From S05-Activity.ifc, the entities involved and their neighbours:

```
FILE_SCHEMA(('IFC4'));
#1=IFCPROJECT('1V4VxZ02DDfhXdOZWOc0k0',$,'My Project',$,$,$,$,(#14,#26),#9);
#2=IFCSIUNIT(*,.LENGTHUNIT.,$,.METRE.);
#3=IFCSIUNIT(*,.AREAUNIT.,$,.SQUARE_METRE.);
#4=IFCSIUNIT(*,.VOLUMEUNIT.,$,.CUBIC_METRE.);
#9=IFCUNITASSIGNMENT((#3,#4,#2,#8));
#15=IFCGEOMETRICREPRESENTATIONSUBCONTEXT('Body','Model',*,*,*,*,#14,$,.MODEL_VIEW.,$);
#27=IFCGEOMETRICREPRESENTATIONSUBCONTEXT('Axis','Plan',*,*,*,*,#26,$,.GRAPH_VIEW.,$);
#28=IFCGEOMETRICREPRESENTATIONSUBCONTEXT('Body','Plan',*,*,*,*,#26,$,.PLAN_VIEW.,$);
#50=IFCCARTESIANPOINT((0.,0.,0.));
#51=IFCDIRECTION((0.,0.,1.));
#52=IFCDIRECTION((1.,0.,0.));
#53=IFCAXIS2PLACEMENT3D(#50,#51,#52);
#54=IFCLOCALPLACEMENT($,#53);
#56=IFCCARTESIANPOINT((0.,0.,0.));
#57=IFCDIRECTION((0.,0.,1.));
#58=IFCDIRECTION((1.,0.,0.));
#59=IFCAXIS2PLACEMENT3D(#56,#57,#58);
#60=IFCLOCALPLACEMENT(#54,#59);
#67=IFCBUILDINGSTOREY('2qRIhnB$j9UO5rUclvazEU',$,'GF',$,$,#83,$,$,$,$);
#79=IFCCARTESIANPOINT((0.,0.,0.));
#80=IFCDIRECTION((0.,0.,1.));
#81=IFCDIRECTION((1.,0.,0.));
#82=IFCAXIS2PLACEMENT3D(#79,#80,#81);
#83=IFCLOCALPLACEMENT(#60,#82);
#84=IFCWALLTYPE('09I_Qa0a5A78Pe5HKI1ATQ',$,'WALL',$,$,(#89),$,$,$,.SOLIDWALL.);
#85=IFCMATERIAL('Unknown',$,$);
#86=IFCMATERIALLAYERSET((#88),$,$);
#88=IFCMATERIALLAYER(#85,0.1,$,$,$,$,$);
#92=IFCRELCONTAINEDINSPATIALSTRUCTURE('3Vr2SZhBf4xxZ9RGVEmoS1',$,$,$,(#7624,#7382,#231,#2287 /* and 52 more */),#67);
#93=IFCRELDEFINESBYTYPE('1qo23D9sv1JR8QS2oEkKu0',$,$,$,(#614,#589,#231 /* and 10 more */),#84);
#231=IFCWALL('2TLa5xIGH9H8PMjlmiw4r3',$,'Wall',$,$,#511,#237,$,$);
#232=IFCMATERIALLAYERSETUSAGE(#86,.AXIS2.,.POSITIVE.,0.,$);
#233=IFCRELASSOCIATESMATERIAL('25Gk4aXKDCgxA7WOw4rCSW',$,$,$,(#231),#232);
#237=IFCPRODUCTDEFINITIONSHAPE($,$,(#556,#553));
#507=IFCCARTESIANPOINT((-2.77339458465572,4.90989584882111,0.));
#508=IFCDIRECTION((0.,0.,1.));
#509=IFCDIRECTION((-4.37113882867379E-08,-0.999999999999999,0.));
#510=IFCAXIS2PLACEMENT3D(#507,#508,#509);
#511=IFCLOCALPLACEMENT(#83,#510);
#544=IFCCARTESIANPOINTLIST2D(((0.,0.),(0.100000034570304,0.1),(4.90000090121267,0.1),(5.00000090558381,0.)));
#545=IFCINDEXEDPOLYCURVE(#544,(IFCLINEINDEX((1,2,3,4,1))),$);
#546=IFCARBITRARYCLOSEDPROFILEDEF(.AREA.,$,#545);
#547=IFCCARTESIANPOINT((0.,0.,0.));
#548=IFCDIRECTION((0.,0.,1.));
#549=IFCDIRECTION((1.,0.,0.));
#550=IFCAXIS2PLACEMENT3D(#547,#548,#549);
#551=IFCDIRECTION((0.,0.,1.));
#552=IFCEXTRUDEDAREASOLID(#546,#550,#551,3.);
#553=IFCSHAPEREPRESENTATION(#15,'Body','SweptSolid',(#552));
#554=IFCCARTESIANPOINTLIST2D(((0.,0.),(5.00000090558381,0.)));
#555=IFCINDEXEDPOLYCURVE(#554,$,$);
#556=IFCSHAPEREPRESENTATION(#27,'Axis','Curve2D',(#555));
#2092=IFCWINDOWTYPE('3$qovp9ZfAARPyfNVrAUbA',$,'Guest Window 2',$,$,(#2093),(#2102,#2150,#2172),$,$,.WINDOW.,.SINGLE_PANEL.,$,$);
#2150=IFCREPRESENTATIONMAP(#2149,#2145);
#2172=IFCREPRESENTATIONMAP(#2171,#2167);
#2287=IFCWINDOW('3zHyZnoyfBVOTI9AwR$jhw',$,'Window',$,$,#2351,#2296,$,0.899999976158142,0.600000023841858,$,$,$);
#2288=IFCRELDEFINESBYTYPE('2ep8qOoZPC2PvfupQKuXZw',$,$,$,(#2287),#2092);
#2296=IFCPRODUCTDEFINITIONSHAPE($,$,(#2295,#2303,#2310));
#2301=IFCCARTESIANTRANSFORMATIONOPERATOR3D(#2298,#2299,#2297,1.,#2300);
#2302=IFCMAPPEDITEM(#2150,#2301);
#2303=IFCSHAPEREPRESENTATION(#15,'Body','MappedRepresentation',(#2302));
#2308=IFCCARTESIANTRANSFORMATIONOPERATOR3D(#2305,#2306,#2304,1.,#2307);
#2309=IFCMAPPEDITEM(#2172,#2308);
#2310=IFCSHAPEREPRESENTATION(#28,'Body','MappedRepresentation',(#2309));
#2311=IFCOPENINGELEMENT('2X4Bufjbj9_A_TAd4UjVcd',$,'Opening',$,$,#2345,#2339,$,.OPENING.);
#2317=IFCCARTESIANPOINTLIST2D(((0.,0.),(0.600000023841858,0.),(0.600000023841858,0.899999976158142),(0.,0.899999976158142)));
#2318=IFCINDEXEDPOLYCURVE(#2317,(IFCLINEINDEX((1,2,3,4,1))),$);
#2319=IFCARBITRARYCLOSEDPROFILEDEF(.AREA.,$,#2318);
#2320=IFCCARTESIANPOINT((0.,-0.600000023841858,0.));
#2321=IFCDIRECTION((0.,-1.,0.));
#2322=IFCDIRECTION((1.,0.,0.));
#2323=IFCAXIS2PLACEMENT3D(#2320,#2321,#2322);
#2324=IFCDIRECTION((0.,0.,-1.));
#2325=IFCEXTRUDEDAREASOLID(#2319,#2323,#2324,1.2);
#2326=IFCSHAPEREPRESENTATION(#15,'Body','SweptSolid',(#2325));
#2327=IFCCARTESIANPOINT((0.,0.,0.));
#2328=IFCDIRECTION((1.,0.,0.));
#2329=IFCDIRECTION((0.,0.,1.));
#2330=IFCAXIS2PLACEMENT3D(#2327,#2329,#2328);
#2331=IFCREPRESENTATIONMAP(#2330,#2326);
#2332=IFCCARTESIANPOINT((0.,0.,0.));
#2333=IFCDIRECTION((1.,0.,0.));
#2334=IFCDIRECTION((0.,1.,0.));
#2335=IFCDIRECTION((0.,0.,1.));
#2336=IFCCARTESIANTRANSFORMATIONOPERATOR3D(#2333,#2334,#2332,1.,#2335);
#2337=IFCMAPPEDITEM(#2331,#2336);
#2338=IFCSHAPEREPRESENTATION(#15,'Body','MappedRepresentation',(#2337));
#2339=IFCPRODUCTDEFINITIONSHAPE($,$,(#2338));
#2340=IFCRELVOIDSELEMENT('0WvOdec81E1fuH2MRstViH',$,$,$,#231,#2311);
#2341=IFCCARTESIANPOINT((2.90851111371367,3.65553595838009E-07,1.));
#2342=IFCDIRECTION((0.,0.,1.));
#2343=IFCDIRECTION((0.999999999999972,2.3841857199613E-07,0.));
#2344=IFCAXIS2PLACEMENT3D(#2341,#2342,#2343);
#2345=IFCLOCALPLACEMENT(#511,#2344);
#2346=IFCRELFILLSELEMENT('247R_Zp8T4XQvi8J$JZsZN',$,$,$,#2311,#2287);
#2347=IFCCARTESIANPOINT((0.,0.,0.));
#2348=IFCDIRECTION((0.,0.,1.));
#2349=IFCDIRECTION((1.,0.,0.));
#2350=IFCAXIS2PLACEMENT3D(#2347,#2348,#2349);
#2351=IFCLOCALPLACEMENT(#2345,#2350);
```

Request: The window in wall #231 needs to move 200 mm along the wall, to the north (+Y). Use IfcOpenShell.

```python
import ifcopenshell
import ifcopenshell.api.geometry
import ifcopenshell.util.placement
import ifcopenshell.util.unit

model = ifcopenshell.open("S05-Activity.ifc")
unit_scale = ifcopenshell.util.unit.calculate_unit_scale(model)

window = model.by_id(2287)
opening = window.FillsVoids[0].RelatingOpeningElement
wall = opening.VoidsElements[0].RelatingBuildingElement

wall_matrix = ifcopenshell.util.placement.get_local_placement(wall.ObjectPlacement)
shift = wall_matrix[:3, 0] * -0.2 / unit_scale
before = ifcopenshell.util.placement.get_local_placement(window.ObjectPlacement)[:3, 3].copy()

# The window is placed relative to its opening, so it follows when the opening moves.
matrix = ifcopenshell.util.placement.get_local_placement(opening.ObjectPlacement)
matrix[:3, 3] += shift
ifcopenshell.api.geometry.edit_object_placement(
    model, product=opening, matrix=matrix, is_si=False, should_transform_children=True
)

after = ifcopenshell.util.placement.get_local_placement(window.ObjectPlacement)[:3, 3]
print("window moved by", (after - before).round(3) + 0.0)

model.write("S05-Activity_v2.ifc")
```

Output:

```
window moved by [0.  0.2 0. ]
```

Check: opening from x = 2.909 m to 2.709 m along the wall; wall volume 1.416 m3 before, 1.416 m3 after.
